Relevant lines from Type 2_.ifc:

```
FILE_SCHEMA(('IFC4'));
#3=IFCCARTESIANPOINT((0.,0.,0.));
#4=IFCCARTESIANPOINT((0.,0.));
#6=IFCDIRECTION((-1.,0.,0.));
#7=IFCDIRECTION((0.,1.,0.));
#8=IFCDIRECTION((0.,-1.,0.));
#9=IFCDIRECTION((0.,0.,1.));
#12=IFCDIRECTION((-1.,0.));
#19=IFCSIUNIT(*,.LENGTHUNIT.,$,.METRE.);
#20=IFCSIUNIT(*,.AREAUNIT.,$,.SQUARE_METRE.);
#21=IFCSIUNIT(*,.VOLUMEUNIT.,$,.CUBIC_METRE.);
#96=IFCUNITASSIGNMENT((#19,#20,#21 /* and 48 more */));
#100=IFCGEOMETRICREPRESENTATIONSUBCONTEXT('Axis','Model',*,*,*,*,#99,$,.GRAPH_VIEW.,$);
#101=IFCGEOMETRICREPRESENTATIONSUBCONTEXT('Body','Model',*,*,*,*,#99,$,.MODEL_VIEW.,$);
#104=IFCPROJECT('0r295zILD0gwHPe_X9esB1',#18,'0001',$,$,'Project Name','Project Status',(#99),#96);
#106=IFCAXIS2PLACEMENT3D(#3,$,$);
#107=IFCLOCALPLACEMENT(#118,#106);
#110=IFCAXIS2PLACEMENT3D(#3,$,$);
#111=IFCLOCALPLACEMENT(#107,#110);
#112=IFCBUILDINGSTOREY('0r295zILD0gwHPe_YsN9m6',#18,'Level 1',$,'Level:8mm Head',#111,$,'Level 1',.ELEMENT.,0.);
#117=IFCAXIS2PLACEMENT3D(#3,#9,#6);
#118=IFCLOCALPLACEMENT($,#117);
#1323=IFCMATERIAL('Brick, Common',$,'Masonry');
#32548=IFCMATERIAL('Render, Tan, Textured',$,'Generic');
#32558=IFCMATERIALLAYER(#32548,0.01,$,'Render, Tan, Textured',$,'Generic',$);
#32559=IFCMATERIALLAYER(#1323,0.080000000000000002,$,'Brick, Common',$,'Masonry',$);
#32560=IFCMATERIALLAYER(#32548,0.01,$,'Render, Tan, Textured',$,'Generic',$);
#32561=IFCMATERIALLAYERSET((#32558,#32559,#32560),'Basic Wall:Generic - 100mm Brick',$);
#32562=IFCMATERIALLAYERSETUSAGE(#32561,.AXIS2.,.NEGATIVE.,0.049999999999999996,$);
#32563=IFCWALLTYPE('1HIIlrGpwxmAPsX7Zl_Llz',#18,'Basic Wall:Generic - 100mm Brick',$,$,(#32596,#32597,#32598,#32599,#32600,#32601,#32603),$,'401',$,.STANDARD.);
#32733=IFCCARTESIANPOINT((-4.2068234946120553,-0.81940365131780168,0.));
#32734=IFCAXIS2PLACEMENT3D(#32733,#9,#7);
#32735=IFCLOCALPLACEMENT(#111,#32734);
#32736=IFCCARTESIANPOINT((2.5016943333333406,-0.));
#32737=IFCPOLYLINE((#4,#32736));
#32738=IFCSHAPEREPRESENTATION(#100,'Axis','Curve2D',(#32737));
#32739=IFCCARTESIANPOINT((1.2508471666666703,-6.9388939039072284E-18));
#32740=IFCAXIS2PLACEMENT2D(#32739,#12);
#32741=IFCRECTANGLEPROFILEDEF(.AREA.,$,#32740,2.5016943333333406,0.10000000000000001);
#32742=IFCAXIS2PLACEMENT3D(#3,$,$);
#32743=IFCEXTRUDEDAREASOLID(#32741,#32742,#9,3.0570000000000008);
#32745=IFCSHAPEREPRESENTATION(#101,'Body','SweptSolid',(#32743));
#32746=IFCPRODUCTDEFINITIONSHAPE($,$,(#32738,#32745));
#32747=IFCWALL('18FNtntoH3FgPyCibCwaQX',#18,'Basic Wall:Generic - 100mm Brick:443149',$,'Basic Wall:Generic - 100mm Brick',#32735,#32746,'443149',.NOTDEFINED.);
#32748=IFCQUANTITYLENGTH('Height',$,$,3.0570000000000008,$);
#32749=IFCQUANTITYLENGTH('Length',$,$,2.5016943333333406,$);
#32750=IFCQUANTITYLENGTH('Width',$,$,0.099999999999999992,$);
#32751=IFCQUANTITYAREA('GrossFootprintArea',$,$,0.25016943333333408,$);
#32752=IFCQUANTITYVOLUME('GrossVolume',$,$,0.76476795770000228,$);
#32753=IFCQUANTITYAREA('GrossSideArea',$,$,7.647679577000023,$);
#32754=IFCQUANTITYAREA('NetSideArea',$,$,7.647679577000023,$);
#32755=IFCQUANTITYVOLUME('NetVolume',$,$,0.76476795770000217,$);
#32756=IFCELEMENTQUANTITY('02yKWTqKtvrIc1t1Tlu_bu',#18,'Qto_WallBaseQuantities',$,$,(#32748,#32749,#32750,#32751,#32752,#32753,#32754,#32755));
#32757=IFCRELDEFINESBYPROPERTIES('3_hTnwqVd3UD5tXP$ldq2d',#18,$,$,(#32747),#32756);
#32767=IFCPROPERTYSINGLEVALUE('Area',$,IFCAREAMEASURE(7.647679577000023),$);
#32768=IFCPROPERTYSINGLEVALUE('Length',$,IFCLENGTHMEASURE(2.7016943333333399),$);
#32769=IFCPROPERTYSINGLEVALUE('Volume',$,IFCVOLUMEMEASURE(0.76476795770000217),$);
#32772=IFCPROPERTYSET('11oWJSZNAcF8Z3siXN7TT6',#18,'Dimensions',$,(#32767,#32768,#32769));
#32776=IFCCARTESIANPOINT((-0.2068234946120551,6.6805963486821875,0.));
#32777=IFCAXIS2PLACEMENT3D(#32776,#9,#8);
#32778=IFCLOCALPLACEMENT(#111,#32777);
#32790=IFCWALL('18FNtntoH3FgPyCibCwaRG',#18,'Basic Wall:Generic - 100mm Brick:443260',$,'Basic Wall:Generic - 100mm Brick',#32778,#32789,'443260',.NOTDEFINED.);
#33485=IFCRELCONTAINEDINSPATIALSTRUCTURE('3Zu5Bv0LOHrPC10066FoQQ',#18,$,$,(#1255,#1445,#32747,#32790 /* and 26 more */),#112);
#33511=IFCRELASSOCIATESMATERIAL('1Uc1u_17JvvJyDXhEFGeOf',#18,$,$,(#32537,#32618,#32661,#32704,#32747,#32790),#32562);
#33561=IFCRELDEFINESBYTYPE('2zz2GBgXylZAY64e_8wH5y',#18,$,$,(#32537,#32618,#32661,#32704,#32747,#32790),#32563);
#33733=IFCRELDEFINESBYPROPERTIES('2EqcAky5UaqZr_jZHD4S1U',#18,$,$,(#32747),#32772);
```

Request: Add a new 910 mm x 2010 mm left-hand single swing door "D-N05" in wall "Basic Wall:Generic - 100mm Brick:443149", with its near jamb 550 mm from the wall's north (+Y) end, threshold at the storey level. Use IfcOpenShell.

```python
import numpy as np
import ifcopenshell
import ifcopenshell.api.feature
import ifcopenshell.api.geometry
import ifcopenshell.api.pset
import ifcopenshell.api.root
import ifcopenshell.api.spatial
import ifcopenshell.geom
import ifcopenshell.util.element
import ifcopenshell.util.placement
import ifcopenshell.util.representation
import ifcopenshell.util.shape
import ifcopenshell.util.unit

model = ifcopenshell.open("Type 2_.ifc")
unit_scale = ifcopenshell.util.unit.calculate_unit_scale(model)
area_scale = ifcopenshell.util.unit.calculate_unit_scale(model, "AREAUNIT")
volume_scale = ifcopenshell.util.unit.calculate_unit_scale(model, "VOLUMEUNIT")
settings = ifcopenshell.geom.settings()


def volume(element):
    """Net volume in cubic metres, openings subtracted."""
    shape = ifcopenshell.geom.create_shape(settings, element)
    return ifcopenshell.util.shape.get_volume(shape.geometry)


wall = model.by_guid("18FNtntoH3FgPyCibCwaQX")
storey = ifcopenshell.util.element.get_container(wall, ifc_class="IfcBuildingStorey")
context = ifcopenshell.util.representation.get_context(model, "Model", "Body", "MODEL_VIEW")
before = volume(wall)

width, height, from_end, sill = 0.91, 2.01, 0.55, 0.0  # metres

# The wall runs along its own X axis, and the end named is its -X end.
wall_shape = ifcopenshell.geom.create_shape(settings, wall)
x, y, z = ifcopenshell.util.shape.get_vertices(wall_shape.geometry).T
start = x.min() + from_end
face, thickness = float(y.min()), float(y.max() - y.min())
wall_matrix = ifcopenshell.util.placement.get_local_placement(wall.ObjectPlacement)
level = ifcopenshell.util.placement.get_local_placement(storey.ObjectPlacement)[2, 3]


def in_wall(x, y):
    """Placement at x, y metres in the wall's axes, at sill height."""
    matrix = wall_matrix.copy()
    matrix[:, 3] = wall_matrix @ np.array([x / unit_scale, y / unit_scale, 0.0, 1.0])
    matrix[2, 3] = level + sill / unit_scale
    return matrix


# Opening: a box that overshoots both wall faces by 50 mm.
opening = ifcopenshell.api.root.create_entity(model, ifc_class="IfcOpeningElement", predefined_type="OPENING")
box = ifcopenshell.api.geometry.add_wall_representation(
    model, context=context, length=width, height=height, thickness=thickness + 0.1
)
ifcopenshell.api.geometry.assign_representation(model, product=opening, representation=box)
ifcopenshell.api.geometry.edit_object_placement(model, product=opening, matrix=in_wall(start, face - 0.05), is_si=False)
ifcopenshell.api.feature.add_feature(model, feature=opening, element=wall)

door = ifcopenshell.api.root.create_entity(model, ifc_class="IfcDoor", name="D-N05", predefined_type="DOOR")
door.OverallWidth, door.OverallHeight = width / unit_scale, height / unit_scale
door.OperationType = "SINGLE_SWING_LEFT"
body = ifcopenshell.api.geometry.add_door_representation(
    model,
    context=context,
    overall_width=door.OverallWidth,
    overall_height=door.OverallHeight,
    operation_type="SINGLE_SWING_LEFT",
    lining_properties={"LiningDepth": thickness / unit_scale, "ThresholdDepth": thickness / unit_scale},
)
ifcopenshell.api.geometry.assign_representation(model, product=door, representation=body)
ifcopenshell.api.spatial.assign_container(model, products=[door], relating_structure=storey)
ifcopenshell.api.feature.add_filling(model, opening=opening, element=door)

# The lining spans the wall, so the door starts at the wall face.
ifcopenshell.api.geometry.edit_object_placement(model, product=door, matrix=in_wall(start, face), is_si=False)

after = volume(wall)

# Update the wall's stored quantities.
qto = model.by_id(ifcopenshell.util.element.get_pset(wall, "Qto_WallBaseQuantities", should_inherit=False)["id"])
ifcopenshell.api.pset.edit_qto(model, qto=qto, properties={
    "NetSideArea": after / thickness / area_scale,
    "NetVolume": after / volume_scale,
})
pset = model.by_id(ifcopenshell.util.element.get_pset(wall, "Dimensions", should_inherit=False)["id"])
ifcopenshell.api.pset.edit_pset(model, pset=pset, properties={
    "Area": model.create_entity("IfcAreaMeasure", after / thickness / area_scale),
    "Volume": model.create_entity("IfcVolumeMeasure", after / volume_scale),
})

print(f"wall volume {before:.3f} -> {after:.3f} m3")

model.write("Type 2_-out.ifc")
```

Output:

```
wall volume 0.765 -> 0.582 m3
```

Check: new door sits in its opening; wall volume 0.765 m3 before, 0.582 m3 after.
